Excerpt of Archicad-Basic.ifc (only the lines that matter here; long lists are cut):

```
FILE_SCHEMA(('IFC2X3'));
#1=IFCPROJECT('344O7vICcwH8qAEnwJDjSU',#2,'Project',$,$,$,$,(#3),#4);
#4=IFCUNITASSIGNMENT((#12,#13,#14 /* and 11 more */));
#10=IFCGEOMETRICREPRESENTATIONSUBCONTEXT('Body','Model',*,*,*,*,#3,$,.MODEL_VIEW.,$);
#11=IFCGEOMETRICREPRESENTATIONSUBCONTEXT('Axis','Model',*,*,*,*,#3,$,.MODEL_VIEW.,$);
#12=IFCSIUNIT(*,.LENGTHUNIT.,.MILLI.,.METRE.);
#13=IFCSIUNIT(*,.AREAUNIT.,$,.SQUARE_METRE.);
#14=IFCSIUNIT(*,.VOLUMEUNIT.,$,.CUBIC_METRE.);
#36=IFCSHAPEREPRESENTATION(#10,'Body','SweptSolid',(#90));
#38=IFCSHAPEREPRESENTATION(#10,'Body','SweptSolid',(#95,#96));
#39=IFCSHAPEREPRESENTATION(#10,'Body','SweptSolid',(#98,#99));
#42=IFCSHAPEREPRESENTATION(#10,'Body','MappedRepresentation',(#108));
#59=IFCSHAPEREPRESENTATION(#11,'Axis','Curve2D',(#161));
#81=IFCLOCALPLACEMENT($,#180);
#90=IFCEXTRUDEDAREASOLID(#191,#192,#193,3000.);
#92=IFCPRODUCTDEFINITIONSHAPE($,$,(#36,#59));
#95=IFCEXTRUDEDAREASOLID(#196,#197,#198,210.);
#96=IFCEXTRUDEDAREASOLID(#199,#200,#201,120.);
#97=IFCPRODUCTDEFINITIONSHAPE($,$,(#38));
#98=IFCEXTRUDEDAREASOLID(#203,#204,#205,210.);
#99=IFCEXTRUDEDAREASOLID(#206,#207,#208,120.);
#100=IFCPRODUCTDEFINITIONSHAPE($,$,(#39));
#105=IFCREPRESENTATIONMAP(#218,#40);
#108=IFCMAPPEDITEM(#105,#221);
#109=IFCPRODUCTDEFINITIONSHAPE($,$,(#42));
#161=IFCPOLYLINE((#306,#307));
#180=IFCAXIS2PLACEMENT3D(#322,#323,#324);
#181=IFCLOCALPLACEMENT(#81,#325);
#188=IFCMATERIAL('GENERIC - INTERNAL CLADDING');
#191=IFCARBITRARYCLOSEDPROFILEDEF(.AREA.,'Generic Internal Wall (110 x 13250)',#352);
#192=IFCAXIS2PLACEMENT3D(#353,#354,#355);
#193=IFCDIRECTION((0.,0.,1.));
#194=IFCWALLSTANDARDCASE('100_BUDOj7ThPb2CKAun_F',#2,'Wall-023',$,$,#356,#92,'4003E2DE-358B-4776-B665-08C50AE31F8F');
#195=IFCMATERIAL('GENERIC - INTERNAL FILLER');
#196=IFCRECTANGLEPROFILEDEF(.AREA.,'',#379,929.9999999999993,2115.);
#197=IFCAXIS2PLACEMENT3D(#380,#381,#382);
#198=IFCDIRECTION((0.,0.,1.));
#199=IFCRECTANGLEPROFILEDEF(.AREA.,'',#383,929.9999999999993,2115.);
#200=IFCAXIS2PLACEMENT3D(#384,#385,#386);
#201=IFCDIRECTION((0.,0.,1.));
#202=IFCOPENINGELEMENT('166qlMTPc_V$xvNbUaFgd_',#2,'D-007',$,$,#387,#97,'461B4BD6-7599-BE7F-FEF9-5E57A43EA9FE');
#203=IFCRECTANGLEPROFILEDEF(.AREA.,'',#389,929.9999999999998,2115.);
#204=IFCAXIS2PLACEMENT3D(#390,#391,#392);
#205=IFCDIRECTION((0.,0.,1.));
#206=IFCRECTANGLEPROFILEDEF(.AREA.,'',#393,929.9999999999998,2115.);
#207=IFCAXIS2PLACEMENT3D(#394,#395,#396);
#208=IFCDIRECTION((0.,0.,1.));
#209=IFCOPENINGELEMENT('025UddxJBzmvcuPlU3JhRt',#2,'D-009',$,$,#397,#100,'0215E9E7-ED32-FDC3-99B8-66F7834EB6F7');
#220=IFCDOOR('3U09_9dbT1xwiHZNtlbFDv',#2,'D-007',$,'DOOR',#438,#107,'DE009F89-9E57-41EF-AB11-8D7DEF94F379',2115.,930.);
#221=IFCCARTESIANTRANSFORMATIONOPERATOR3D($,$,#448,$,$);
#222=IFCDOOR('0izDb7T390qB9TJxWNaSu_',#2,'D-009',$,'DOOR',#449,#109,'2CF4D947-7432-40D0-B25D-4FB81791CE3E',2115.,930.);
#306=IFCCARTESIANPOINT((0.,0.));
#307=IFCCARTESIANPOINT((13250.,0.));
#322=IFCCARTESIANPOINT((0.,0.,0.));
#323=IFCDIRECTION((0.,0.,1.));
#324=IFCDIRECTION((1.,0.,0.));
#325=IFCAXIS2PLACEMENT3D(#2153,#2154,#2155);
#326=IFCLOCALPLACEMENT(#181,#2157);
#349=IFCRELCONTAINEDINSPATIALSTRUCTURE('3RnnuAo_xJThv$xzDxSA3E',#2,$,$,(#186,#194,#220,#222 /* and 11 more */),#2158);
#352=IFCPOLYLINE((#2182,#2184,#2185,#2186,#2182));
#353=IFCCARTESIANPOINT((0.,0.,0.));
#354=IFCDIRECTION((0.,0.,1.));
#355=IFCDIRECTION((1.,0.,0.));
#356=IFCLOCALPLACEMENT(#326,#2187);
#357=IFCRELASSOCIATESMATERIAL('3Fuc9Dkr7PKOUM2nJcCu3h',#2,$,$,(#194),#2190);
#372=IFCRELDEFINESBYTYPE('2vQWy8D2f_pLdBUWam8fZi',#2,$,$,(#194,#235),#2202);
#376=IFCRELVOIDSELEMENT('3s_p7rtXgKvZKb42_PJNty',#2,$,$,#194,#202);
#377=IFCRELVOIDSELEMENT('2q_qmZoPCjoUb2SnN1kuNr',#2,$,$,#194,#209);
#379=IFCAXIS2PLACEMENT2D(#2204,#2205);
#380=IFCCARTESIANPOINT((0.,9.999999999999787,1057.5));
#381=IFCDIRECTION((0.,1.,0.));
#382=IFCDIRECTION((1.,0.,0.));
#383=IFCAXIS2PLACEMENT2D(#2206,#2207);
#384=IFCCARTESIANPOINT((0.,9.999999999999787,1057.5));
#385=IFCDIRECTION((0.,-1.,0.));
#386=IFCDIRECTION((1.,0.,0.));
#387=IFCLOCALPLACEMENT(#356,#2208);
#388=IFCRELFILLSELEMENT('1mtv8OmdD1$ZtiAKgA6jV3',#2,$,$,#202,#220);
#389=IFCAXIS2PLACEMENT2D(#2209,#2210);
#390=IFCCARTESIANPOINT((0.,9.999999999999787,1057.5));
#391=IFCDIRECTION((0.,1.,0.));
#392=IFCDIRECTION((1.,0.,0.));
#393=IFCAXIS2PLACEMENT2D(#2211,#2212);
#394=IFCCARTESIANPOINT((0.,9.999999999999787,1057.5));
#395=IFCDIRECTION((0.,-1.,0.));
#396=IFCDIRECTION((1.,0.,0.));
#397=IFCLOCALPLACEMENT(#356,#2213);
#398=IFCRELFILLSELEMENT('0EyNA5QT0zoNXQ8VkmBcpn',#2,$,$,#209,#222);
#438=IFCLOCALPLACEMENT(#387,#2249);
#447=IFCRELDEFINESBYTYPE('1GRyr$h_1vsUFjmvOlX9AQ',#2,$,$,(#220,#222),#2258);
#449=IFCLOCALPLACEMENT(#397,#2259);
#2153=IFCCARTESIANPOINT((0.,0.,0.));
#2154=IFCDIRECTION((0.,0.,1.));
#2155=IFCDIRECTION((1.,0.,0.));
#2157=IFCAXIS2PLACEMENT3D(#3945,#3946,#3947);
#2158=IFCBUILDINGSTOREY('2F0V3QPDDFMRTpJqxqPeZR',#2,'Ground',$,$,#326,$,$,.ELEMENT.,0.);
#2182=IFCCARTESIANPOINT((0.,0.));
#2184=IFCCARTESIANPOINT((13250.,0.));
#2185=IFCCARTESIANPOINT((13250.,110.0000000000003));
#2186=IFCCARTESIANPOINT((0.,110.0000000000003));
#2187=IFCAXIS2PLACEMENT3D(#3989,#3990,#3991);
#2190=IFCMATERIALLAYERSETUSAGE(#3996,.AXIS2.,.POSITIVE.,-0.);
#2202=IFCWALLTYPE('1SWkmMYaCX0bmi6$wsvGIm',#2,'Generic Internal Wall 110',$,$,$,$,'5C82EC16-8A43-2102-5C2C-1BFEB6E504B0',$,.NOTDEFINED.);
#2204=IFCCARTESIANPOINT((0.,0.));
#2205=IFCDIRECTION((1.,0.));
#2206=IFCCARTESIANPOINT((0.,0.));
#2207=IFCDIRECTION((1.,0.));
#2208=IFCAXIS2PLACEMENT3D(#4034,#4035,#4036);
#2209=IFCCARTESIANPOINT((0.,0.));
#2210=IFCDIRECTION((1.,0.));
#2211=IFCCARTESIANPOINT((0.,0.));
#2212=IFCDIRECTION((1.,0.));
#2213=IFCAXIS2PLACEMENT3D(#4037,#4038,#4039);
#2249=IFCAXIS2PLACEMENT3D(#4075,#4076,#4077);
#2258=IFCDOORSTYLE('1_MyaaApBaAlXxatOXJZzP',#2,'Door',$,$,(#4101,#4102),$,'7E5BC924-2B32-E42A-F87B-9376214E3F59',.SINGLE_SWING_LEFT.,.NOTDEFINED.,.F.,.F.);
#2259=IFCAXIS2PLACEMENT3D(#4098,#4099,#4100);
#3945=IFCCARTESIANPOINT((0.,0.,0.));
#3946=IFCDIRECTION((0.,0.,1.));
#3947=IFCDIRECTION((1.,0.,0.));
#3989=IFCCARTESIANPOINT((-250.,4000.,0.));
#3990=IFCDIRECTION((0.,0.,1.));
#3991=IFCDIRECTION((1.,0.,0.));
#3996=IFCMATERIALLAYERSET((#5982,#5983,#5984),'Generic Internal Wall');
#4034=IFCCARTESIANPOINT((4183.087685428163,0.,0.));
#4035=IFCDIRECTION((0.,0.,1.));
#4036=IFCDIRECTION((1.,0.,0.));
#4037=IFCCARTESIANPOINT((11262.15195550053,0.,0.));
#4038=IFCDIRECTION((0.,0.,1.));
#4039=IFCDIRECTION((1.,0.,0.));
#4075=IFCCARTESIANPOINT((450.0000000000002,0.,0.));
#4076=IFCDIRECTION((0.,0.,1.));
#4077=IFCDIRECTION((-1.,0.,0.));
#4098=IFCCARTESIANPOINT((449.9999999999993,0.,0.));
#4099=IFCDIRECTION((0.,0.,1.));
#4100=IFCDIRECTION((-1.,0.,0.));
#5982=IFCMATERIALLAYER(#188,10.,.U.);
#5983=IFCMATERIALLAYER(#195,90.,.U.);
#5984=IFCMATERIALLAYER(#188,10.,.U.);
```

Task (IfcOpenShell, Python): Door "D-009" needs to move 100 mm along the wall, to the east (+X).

```python
import ifcopenshell
import ifcopenshell.api.geometry
import ifcopenshell.util.placement
import ifcopenshell.util.unit

model = ifcopenshell.open("Archicad-Basic.ifc")
unit_scale = ifcopenshell.util.unit.calculate_unit_scale(model)

door = model.by_guid("0izDb7T390qB9TJxWNaSu_")
opening = door.FillsVoids[0].RelatingOpeningElement
wall = opening.VoidsElements[0].RelatingBuildingElement

wall_matrix = ifcopenshell.util.placement.get_local_placement(wall.ObjectPlacement)
shift = wall_matrix[:3, 0] * 0.1 / unit_scale
before = ifcopenshell.util.placement.get_local_placement(door.ObjectPlacement)[:3, 3].copy()

# The door is placed relative to its opening, so it follows when the opening moves.
matrix = ifcopenshell.util.placement.get_local_placement(opening.ObjectPlacement)
matrix[:3, 3] += shift
ifcopenshell.api.geometry.edit_object_placement(
    model, product=opening, matrix=matrix, is_si=False, should_transform_children=True
)

after = ifcopenshell.util.placement.get_local_placement(door.ObjectPlacement)[:3, 3]
print("door moved by", (after - before).round(3) + 0.0)

model.write("Archicad-Basic_edited.ifc")
```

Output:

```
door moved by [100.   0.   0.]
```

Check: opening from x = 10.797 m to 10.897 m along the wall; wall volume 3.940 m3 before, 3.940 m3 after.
